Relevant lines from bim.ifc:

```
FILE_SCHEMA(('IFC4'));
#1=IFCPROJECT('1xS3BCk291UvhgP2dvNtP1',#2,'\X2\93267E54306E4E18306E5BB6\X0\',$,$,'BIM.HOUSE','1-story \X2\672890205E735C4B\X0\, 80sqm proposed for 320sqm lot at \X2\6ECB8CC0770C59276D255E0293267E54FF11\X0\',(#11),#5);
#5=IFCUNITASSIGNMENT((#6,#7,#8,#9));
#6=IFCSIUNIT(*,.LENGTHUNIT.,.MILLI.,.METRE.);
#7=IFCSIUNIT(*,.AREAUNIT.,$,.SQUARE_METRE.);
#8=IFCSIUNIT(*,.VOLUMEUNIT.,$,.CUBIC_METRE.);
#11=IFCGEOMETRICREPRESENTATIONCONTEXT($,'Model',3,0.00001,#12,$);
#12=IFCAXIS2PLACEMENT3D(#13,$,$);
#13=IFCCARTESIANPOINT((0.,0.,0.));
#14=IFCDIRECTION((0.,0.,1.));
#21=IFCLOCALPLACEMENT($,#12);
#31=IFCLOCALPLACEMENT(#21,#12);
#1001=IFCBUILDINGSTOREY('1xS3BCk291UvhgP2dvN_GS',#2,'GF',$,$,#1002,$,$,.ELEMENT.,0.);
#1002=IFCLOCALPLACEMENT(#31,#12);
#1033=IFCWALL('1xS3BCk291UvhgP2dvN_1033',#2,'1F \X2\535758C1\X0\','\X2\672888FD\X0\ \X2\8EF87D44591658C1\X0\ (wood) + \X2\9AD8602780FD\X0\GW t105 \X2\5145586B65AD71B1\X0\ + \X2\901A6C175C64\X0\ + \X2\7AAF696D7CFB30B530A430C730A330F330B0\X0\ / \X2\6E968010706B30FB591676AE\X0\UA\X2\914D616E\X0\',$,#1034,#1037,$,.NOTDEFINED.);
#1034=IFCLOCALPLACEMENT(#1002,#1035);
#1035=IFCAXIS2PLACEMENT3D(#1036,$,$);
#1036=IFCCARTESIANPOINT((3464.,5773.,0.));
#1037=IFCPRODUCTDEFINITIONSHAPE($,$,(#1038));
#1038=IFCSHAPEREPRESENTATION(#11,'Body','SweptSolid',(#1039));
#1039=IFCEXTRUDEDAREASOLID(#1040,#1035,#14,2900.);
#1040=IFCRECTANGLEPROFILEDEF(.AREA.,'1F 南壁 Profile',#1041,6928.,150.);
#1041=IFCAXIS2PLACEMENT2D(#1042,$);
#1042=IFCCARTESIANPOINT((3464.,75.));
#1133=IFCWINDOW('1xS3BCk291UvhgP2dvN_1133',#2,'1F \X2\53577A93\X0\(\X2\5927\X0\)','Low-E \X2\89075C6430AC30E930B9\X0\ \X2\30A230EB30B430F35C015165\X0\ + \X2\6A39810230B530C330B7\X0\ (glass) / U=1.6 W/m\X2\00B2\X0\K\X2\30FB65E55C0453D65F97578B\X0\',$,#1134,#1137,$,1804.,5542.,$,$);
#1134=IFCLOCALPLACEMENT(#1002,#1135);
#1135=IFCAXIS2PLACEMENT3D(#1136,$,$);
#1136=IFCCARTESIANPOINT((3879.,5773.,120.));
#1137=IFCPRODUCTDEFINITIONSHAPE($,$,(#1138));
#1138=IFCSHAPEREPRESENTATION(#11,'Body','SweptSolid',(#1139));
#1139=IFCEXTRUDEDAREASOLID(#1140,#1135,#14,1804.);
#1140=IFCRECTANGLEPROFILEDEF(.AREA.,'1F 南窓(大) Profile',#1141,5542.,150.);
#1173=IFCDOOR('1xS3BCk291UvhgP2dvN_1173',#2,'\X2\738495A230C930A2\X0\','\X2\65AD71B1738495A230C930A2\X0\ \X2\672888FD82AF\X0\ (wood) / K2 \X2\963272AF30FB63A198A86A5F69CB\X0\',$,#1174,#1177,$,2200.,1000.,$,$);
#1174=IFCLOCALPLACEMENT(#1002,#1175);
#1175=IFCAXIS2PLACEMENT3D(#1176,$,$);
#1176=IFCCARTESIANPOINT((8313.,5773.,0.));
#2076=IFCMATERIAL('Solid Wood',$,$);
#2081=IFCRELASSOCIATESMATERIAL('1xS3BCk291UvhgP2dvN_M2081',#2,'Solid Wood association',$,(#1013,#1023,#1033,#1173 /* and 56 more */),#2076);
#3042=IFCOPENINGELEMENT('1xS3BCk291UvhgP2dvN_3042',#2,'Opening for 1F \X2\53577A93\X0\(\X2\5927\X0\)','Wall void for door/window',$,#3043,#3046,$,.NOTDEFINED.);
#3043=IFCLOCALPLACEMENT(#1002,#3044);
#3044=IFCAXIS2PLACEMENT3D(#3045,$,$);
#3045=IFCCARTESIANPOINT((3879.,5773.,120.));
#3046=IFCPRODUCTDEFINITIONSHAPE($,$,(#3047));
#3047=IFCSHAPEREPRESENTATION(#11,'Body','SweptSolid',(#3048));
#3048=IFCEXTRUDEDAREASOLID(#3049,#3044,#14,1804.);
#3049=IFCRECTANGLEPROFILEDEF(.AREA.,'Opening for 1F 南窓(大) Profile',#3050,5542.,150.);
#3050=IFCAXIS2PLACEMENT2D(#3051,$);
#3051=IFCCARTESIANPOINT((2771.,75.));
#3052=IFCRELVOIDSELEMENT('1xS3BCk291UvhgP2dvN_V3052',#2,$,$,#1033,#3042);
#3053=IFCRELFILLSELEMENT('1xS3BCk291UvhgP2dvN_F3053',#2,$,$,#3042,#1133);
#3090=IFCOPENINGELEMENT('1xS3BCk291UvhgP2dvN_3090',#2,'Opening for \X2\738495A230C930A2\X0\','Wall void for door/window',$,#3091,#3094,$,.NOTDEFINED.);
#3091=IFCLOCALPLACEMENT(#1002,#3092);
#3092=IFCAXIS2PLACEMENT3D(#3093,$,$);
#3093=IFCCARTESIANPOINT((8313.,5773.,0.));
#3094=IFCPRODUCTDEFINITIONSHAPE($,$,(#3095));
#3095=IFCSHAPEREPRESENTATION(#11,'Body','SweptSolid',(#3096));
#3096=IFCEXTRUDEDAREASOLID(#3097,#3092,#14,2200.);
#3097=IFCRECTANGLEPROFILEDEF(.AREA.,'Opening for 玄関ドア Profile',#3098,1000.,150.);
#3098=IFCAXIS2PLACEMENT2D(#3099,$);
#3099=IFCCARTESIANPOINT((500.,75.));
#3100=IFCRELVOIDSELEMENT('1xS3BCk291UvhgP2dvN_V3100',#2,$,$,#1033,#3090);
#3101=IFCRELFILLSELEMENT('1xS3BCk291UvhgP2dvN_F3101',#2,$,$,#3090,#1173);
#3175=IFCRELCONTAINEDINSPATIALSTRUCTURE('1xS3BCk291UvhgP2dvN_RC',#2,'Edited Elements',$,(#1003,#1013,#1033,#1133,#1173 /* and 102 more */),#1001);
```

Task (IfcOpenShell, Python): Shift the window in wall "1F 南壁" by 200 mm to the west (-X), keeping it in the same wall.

```python
import ifcopenshell
import ifcopenshell.api.geometry
import ifcopenshell.util.placement

model = ifcopenshell.open("bim.ifc")

window = model.by_guid("1xS3BCk291UvhgP2dvN_1133")
opening = window.FillsVoids[0].RelatingOpeningElement
wall = opening.VoidsElements[0].RelatingBuildingElement

wall_matrix = ifcopenshell.util.placement.get_local_placement(wall.ObjectPlacement)
shift = wall_matrix[:3, 0] * -200.0
before = ifcopenshell.util.placement.get_local_placement(window.ObjectPlacement)[:3, 3].copy()

# The window is not placed relative to its opening, so move both.
for product in (opening, window):
    matrix = ifcopenshell.util.placement.get_local_placement(product.ObjectPlacement)
    matrix[:3, 3] += shift
    ifcopenshell.api.geometry.edit_object_placement(model, product=product, matrix=matrix, is_si=False)

after = ifcopenshell.util.placement.get_local_placement(window.ObjectPlacement)[:3, 3]
print("window moved by", (after - before).round(3) + 0.0)

model.write("bim_updated.ifc")
```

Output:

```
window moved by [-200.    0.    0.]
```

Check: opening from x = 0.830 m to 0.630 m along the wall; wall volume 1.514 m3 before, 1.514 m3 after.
